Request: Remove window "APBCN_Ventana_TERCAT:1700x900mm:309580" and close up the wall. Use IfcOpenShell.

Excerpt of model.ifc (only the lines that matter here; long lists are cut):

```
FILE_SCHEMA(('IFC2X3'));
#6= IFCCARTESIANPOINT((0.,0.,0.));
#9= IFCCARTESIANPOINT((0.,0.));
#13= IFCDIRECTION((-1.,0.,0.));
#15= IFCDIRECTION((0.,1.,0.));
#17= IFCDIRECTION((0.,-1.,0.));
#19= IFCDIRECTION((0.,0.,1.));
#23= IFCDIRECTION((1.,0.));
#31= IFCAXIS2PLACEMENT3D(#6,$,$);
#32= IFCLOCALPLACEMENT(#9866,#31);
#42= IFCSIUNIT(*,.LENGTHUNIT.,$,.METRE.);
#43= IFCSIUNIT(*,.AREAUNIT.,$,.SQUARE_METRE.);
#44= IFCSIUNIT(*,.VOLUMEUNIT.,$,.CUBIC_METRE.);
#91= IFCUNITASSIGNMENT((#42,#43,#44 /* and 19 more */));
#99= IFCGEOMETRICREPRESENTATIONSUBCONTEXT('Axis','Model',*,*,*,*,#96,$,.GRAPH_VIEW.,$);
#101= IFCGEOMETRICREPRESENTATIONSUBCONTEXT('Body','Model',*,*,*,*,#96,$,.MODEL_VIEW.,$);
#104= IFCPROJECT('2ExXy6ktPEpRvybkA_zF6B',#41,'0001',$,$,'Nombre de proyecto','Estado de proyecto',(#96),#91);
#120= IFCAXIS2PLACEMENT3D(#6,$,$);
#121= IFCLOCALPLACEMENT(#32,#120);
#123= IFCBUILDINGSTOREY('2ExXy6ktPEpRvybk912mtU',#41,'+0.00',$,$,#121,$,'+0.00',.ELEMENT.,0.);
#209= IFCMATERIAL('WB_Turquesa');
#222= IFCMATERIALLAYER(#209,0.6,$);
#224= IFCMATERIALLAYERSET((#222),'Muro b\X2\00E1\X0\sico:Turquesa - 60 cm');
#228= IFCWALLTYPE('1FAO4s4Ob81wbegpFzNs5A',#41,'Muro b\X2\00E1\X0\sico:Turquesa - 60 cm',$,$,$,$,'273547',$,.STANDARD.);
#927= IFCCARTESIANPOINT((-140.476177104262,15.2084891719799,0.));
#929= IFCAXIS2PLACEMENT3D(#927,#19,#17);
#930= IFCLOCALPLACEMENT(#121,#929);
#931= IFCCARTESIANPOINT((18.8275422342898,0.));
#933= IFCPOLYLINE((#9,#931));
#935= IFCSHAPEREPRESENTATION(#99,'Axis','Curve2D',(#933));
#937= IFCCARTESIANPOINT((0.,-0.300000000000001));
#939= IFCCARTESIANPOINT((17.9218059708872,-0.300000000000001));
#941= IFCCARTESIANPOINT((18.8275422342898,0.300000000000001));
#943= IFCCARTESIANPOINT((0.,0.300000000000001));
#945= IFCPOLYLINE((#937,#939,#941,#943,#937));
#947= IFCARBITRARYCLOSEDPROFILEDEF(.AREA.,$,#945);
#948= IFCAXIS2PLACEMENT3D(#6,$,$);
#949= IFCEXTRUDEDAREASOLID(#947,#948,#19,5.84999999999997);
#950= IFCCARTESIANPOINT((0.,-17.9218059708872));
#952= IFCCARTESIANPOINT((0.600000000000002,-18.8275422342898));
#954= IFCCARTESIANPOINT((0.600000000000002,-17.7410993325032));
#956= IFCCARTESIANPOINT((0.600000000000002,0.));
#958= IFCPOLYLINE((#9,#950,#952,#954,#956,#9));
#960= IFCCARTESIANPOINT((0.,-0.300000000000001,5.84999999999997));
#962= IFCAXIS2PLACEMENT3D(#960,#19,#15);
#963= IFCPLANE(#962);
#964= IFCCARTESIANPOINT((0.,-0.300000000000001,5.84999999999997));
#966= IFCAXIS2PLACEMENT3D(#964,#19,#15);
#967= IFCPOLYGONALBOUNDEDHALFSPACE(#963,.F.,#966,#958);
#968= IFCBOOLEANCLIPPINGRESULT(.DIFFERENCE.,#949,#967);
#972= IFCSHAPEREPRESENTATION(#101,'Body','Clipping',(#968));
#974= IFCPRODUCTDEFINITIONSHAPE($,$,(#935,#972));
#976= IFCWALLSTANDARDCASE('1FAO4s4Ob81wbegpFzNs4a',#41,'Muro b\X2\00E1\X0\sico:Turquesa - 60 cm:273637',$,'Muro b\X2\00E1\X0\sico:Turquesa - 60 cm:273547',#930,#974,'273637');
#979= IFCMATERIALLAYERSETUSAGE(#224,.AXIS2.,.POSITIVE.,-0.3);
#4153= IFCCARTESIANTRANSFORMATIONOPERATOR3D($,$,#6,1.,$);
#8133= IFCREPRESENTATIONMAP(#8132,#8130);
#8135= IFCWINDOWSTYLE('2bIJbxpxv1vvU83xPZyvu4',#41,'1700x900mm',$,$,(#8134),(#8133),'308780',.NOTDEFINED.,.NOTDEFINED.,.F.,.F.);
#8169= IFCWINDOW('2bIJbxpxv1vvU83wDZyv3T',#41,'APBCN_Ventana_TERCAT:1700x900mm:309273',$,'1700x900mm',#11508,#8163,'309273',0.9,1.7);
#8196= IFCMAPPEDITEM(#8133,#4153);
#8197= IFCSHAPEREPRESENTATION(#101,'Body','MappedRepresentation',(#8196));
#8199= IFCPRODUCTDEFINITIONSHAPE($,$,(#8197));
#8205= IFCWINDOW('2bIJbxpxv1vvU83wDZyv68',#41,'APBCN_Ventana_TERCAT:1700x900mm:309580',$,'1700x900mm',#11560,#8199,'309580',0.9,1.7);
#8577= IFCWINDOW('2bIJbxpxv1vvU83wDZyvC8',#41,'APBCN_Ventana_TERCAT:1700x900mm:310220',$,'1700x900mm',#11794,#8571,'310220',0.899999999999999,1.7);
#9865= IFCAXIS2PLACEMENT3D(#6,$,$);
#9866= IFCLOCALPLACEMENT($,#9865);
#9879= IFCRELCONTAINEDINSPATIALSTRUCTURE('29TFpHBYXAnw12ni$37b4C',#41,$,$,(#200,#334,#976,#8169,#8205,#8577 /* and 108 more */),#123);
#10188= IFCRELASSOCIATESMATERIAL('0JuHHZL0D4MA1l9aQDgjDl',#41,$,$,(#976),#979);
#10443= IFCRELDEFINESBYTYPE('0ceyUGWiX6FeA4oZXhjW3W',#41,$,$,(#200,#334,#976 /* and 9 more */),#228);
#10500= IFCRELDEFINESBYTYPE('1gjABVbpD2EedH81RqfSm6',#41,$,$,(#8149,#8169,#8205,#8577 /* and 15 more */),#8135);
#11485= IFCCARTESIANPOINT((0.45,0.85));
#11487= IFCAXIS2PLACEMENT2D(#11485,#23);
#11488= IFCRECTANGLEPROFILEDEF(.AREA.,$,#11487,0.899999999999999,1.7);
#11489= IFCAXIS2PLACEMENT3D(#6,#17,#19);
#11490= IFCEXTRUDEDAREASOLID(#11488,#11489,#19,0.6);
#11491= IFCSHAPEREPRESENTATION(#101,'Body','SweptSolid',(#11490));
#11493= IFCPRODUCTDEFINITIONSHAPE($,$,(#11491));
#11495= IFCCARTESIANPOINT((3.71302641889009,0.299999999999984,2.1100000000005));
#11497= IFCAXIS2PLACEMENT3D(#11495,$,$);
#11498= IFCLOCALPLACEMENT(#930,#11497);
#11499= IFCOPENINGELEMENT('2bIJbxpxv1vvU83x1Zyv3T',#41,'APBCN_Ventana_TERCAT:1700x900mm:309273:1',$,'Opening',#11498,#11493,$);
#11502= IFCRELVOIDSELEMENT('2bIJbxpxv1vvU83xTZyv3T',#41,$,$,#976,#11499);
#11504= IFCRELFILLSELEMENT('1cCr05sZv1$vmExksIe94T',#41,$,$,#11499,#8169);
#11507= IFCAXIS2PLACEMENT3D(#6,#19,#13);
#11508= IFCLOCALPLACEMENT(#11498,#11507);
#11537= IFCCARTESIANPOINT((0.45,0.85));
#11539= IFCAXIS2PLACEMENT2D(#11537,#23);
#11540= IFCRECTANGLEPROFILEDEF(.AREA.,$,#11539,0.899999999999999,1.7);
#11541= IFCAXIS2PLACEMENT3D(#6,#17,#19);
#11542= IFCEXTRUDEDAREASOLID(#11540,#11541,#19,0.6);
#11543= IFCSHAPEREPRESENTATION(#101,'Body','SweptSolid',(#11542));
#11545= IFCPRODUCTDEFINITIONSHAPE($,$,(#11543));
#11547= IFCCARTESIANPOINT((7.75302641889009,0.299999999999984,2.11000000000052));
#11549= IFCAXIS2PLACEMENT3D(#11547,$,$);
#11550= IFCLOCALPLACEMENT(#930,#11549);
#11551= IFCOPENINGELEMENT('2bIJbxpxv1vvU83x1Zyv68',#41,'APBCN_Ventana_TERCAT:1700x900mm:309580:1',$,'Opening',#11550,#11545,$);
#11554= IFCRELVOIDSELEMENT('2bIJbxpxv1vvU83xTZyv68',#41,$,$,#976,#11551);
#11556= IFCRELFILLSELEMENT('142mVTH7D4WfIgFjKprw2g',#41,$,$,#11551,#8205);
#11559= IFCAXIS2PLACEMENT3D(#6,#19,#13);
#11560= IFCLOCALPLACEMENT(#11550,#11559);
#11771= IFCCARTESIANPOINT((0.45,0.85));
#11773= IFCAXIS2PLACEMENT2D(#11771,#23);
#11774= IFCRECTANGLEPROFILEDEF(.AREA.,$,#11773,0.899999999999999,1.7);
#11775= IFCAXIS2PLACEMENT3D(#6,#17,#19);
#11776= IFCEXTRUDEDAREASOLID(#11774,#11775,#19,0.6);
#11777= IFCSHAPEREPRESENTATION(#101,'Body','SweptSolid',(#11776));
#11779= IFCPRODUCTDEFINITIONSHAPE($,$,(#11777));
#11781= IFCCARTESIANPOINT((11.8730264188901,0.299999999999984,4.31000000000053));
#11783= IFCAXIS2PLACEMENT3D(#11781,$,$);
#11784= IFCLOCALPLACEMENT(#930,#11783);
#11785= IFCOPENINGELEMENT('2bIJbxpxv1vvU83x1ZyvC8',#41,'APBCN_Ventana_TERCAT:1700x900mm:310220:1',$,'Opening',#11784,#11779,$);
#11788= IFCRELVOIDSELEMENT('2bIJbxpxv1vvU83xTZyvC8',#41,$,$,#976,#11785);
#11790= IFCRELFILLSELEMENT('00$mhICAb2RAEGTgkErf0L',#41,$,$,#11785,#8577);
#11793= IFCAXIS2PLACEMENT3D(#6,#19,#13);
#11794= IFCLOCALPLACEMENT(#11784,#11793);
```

```python
import ifcopenshell
import ifcopenshell.api.feature
import ifcopenshell.api.root
import ifcopenshell.geom
import ifcopenshell.util.shape

model = ifcopenshell.open("model.ifc")
settings = ifcopenshell.geom.settings()


def volume(element):
    """Net volume in cubic metres, openings subtracted."""
    shape = ifcopenshell.geom.create_shape(settings, element)
    return ifcopenshell.util.shape.get_volume(shape.geometry)


window = model.by_guid("2bIJbxpxv1vvU83wDZyv68")
opening = window.FillsVoids[0].RelatingOpeningElement
wall = opening.VoidsElements[0].RelatingBuildingElement
before = volume(wall)

ifcopenshell.api.root.remove_product(model, product=window)
ifcopenshell.api.feature.remove_feature(model, feature=opening)

after = volume(wall)

print(f"wall volume {before:.3f} -> {after:.3f} m3")

model.write("model-out.ifc")
```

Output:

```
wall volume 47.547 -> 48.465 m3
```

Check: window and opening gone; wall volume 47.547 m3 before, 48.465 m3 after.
